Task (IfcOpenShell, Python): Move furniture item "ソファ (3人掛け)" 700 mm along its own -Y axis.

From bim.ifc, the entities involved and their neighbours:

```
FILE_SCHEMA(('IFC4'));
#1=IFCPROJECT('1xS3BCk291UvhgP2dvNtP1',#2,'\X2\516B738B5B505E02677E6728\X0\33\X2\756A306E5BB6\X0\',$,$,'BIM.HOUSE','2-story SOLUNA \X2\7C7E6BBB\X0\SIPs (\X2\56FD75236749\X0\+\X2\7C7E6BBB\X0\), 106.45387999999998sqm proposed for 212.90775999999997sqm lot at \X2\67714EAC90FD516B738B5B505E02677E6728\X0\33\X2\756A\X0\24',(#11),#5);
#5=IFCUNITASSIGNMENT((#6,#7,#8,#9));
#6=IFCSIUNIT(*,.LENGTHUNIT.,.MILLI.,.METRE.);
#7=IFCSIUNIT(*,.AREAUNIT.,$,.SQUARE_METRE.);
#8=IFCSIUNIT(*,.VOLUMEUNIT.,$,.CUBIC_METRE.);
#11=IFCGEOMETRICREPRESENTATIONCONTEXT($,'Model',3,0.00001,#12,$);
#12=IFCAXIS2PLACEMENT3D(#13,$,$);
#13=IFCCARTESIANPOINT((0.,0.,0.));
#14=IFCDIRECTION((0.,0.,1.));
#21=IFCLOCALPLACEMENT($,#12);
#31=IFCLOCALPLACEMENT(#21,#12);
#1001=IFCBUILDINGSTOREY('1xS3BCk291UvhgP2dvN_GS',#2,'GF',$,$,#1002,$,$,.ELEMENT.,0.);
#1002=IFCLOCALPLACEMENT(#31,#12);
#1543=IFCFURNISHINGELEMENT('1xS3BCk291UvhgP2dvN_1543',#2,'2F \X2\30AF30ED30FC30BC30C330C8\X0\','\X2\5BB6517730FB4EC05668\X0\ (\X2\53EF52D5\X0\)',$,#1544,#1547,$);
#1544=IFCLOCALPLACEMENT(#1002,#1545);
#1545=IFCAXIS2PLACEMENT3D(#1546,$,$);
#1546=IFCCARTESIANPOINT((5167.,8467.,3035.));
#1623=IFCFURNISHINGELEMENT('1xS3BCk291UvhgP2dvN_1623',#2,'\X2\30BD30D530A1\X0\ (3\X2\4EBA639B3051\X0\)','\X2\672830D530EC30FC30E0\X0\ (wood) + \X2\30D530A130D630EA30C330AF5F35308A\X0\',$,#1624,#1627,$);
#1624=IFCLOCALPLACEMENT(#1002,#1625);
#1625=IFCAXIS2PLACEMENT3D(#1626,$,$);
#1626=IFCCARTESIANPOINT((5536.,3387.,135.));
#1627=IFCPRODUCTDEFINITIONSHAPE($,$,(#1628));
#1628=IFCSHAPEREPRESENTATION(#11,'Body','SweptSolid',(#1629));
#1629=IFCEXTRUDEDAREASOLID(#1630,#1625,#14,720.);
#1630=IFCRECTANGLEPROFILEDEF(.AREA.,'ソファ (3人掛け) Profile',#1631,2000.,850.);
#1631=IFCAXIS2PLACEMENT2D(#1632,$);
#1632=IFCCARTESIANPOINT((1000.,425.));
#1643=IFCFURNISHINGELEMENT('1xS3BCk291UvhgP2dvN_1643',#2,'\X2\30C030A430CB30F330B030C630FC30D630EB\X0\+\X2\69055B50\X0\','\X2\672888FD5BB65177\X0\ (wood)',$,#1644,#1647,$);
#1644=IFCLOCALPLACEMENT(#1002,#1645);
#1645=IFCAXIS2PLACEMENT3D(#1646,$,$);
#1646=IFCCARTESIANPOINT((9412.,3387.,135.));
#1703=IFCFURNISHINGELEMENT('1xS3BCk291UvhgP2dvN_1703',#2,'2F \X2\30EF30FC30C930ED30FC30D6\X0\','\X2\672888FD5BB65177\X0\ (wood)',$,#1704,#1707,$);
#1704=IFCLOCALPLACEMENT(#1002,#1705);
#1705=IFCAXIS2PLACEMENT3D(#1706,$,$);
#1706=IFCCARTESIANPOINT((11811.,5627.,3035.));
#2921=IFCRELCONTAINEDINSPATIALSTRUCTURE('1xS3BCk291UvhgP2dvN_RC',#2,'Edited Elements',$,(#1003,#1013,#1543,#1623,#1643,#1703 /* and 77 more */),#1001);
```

```python
import ifcopenshell
import ifcopenshell.api.geometry
import ifcopenshell.util.placement

model = ifcopenshell.open("bim.ifc")

item = model.by_guid("1xS3BCk291UvhgP2dvN_1623")
matrix = ifcopenshell.util.placement.get_local_placement(item.ObjectPlacement)
matrix[:3, 3] -= matrix[:3, 1] * 700.0
ifcopenshell.api.geometry.edit_object_placement(model, product=item, matrix=matrix, is_si=False)

print(ifcopenshell.util.placement.get_local_placement(item.ObjectPlacement).round(3) + 0.0)

model.write("bim_updated.ifc")
```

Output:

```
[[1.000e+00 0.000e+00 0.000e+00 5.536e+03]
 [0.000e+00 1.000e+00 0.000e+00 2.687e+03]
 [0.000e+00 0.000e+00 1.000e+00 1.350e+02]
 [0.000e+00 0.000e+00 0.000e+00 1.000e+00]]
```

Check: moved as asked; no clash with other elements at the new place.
